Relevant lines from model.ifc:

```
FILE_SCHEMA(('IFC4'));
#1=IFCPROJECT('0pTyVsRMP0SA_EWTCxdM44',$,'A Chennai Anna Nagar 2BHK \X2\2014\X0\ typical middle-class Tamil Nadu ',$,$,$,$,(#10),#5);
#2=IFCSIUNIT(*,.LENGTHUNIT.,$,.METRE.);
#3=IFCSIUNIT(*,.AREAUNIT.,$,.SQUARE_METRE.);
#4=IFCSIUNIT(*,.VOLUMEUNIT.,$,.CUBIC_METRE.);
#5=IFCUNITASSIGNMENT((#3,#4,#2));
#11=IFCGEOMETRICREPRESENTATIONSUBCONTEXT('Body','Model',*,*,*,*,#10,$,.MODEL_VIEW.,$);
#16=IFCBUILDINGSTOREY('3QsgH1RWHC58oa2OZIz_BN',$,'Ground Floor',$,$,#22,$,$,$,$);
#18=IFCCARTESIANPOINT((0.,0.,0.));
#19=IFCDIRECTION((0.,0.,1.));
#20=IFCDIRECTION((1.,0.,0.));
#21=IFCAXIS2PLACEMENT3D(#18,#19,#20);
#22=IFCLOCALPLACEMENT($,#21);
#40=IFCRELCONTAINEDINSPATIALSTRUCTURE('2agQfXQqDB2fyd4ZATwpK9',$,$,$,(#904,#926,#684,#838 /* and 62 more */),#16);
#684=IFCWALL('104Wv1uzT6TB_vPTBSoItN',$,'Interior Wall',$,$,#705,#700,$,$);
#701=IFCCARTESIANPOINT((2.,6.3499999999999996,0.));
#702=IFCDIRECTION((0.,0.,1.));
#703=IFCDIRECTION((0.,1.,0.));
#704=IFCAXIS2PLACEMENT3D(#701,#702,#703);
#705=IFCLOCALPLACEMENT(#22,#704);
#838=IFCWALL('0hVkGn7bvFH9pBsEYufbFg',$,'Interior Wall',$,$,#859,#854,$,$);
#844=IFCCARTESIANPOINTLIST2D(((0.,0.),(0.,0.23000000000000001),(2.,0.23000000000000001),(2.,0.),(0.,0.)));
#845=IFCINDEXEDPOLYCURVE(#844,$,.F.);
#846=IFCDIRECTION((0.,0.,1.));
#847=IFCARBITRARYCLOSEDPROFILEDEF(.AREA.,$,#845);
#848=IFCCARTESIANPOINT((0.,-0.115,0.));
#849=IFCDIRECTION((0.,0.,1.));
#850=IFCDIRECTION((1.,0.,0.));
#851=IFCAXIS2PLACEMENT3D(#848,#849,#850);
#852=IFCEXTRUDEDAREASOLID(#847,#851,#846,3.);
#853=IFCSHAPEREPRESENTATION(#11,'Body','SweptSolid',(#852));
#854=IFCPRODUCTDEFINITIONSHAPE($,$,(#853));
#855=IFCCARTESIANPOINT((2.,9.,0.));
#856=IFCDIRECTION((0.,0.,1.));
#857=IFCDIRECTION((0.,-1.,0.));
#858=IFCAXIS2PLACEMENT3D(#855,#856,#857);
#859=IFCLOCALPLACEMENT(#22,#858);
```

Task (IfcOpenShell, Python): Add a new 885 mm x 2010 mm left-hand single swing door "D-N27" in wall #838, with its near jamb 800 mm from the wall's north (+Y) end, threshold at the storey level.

```python
import numpy as np
import ifcopenshell
import ifcopenshell.api.feature
import ifcopenshell.api.geometry
import ifcopenshell.api.root
import ifcopenshell.api.spatial
import ifcopenshell.geom
import ifcopenshell.util.element
import ifcopenshell.util.placement
import ifcopenshell.util.representation
import ifcopenshell.util.shape
import ifcopenshell.util.unit

model = ifcopenshell.open("model.ifc")
unit_scale = ifcopenshell.util.unit.calculate_unit_scale(model)
settings = ifcopenshell.geom.settings()


def volume(element):
    """Net volume in cubic metres, openings subtracted."""
    shape = ifcopenshell.geom.create_shape(settings, element)
    return ifcopenshell.util.shape.get_volume(shape.geometry)


wall = model.by_guid("0hVkGn7bvFH9pBsEYufbFg")
storey = ifcopenshell.util.element.get_container(wall, ifc_class="IfcBuildingStorey")
context = ifcopenshell.util.representation.get_context(model, "Model", "Body", "MODEL_VIEW")
before = volume(wall)

width, height, from_end, sill = 0.885, 2.01, 0.8, 0.0  # metres

# The wall runs along its own X axis, and the end named is its -X end.
wall_shape = ifcopenshell.geom.create_shape(settings, wall)
x, y, z = ifcopenshell.util.shape.get_vertices(wall_shape.geometry).T
start = x.min() + from_end
face, thickness = float(y.min()), float(y.max() - y.min())
wall_matrix = ifcopenshell.util.placement.get_local_placement(wall.ObjectPlacement)
level = ifcopenshell.util.placement.get_local_placement(storey.ObjectPlacement)[2, 3]


def in_wall(x, y):
    """Placement at x, y metres in the wall's axes, at sill height."""
    matrix = wall_matrix.copy()
    matrix[:, 3] = wall_matrix @ np.array([x / unit_scale, y / unit_scale, 0.0, 1.0])
    matrix[2, 3] = level + sill / unit_scale
    return matrix


# Opening: a box that overshoots both wall faces by 50 mm.
opening = ifcopenshell.api.root.create_entity(model, ifc_class="IfcOpeningElement", predefined_type="OPENING")
box = ifcopenshell.api.geometry.add_wall_representation(
    model, context=context, length=width, height=height, thickness=thickness + 0.1
)
ifcopenshell.api.geometry.assign_representation(model, product=opening, representation=box)
ifcopenshell.api.geometry.edit_object_placement(model, product=opening, matrix=in_wall(start, face - 0.05), is_si=False)
ifcopenshell.api.feature.add_feature(model, feature=opening, element=wall)

door = ifcopenshell.api.root.create_entity(model, ifc_class="IfcDoor", name="D-N27", predefined_type="DOOR")
door.OverallWidth, door.OverallHeight = width / unit_scale, height / unit_scale
door.OperationType = "SINGLE_SWING_LEFT"
body = ifcopenshell.api.geometry.add_door_representation(
    model,
    context=context,
    overall_width=door.OverallWidth,
    overall_height=door.OverallHeight,
    operation_type="SINGLE_SWING_LEFT",
    lining_properties={"LiningDepth": thickness / unit_scale, "ThresholdDepth": thickness / unit_scale},
)
ifcopenshell.api.geometry.assign_representation(model, product=door, representation=body)
ifcopenshell.api.spatial.assign_container(model, products=[door], relating_structure=storey)
ifcopenshell.api.feature.add_filling(model, opening=opening, element=door)

# The lining spans the wall, so the door starts at the wall face.
ifcopenshell.api.geometry.edit_object_placement(model, product=door, matrix=in_wall(start, face), is_si=False)

after = volume(wall)

print(f"wall volume {before:.3f} -> {after:.3f} m3")

model.write("model_edited.ifc")
```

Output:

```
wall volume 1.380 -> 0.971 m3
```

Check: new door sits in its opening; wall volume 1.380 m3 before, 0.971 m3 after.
